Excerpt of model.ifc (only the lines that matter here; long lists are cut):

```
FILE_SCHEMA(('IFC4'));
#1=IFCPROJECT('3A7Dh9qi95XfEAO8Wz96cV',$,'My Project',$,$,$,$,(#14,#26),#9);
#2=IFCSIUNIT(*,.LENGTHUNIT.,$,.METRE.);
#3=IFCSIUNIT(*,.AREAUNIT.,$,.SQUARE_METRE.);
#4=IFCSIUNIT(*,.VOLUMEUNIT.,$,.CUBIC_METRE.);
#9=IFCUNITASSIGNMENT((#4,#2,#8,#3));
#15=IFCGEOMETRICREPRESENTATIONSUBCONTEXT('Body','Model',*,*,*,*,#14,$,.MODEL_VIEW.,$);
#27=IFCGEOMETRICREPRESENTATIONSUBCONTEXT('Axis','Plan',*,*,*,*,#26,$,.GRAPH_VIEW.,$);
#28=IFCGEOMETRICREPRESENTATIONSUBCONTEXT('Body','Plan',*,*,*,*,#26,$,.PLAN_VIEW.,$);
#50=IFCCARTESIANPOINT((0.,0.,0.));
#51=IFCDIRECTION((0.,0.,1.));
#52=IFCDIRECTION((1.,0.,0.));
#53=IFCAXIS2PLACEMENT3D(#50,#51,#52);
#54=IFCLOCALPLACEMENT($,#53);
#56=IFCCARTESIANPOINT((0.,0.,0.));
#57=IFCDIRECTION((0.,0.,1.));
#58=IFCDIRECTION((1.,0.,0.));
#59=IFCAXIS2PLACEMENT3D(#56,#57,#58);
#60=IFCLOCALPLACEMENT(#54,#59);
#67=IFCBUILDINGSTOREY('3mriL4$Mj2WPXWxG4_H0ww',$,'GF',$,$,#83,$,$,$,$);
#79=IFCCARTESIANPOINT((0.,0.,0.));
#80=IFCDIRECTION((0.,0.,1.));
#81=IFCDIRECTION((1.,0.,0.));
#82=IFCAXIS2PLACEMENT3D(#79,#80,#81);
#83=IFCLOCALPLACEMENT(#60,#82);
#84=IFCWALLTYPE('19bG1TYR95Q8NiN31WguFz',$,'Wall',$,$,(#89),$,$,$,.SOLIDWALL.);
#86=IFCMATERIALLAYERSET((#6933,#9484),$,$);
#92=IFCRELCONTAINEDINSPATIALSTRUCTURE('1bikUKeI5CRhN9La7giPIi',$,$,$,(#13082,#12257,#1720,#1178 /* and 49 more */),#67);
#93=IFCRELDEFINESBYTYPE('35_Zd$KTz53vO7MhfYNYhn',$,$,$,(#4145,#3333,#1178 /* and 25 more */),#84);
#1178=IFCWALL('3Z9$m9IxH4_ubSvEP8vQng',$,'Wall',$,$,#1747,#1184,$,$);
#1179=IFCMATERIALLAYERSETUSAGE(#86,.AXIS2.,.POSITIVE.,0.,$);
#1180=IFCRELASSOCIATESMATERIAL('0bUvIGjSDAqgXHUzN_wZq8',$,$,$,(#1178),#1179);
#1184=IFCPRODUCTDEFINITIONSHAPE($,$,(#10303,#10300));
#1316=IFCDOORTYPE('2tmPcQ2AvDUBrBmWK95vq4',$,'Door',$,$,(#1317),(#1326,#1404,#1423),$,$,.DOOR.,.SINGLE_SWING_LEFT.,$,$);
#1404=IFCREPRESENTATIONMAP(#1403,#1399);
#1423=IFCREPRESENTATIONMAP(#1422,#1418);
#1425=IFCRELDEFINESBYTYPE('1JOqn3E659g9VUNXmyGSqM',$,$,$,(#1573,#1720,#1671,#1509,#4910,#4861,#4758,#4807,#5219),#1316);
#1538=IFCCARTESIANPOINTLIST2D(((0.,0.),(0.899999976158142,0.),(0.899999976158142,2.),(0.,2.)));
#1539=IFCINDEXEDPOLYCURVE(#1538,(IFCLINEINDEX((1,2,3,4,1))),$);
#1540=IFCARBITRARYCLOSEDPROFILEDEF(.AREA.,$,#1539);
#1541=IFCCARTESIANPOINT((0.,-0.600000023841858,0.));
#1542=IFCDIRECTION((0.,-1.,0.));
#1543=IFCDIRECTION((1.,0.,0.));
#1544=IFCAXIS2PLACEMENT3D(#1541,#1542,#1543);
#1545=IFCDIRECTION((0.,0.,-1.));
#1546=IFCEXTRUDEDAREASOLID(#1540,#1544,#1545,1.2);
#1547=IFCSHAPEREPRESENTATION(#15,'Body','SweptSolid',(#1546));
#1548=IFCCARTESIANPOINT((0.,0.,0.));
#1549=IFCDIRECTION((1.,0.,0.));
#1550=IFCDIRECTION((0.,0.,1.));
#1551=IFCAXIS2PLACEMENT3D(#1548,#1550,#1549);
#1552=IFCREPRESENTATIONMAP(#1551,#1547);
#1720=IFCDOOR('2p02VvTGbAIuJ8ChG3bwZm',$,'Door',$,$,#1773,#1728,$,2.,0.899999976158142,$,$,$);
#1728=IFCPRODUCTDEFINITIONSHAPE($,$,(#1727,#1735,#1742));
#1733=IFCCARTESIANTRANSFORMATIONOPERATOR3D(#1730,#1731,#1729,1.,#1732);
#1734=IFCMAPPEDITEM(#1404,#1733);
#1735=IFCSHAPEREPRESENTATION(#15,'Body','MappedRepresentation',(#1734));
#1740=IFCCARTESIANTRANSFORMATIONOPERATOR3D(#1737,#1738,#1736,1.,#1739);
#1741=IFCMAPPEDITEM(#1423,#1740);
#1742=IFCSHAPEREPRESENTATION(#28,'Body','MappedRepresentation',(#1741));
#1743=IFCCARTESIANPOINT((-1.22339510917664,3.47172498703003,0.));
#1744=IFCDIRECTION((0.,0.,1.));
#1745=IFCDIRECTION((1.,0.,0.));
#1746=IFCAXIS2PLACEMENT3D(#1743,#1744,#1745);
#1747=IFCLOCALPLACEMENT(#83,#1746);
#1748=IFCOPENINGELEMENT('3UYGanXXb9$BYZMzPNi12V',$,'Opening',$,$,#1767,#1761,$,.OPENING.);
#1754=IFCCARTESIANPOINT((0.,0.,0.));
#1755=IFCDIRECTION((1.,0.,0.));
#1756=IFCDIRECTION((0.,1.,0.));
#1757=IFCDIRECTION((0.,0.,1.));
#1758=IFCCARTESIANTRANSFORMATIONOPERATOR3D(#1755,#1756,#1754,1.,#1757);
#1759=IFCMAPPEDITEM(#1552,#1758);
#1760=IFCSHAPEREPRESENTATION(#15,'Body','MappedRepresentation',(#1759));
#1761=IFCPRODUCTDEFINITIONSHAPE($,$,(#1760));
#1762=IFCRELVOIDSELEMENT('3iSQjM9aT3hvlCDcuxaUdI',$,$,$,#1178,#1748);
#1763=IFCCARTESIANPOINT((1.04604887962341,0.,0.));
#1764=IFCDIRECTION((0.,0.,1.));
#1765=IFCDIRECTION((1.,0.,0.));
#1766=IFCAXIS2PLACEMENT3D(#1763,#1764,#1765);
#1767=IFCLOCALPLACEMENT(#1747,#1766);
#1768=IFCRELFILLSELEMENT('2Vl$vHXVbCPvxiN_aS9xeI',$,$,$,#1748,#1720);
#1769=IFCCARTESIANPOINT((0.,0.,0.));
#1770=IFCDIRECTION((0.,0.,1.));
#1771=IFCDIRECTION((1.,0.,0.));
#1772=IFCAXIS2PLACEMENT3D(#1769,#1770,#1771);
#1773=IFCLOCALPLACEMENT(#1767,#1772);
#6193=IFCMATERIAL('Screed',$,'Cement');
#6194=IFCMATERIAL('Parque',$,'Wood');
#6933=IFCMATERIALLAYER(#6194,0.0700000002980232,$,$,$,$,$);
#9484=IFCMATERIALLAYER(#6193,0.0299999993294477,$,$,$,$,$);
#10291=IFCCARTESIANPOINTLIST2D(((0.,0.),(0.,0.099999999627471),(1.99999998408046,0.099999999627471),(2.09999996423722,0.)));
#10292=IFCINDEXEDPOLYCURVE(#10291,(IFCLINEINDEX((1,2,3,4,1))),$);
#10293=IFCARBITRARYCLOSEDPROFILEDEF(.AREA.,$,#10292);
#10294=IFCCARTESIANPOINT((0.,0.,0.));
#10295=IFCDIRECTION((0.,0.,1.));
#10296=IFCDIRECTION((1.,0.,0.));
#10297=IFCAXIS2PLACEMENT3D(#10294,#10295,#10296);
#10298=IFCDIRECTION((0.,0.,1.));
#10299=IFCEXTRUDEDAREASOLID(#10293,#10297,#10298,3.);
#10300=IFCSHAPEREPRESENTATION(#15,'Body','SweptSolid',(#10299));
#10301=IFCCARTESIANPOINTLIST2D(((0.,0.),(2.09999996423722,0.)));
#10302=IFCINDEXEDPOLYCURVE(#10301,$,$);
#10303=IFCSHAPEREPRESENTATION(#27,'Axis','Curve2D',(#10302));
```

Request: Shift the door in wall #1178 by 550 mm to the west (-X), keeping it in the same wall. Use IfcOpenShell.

```python
import ifcopenshell
import ifcopenshell.api.geometry
import ifcopenshell.util.placement
import ifcopenshell.util.unit

model = ifcopenshell.open("model.ifc")
unit_scale = ifcopenshell.util.unit.calculate_unit_scale(model)

door = model.by_guid("2p02VvTGbAIuJ8ChG3bwZm")
opening = door.FillsVoids[0].RelatingOpeningElement
wall = opening.VoidsElements[0].RelatingBuildingElement

wall_matrix = ifcopenshell.util.placement.get_local_placement(wall.ObjectPlacement)
shift = wall_matrix[:3, 0] * -0.55 / unit_scale
before = ifcopenshell.util.placement.get_local_placement(door.ObjectPlacement)[:3, 3].copy()

# The door is placed relative to its opening, so it follows when the opening moves.
matrix = ifcopenshell.util.placement.get_local_placement(opening.ObjectPlacement)
matrix[:3, 3] += shift
ifcopenshell.api.geometry.edit_object_placement(
    model, product=opening, matrix=matrix, is_si=False, should_transform_children=True
)

after = ifcopenshell.util.placement.get_local_placement(door.ObjectPlacement)[:3, 3]
print("door moved by", (after - before).round(3) + 0.0)

model.write("model_updated.ifc")
```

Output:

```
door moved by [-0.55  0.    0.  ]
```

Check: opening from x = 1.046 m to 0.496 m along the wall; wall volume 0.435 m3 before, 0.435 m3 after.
